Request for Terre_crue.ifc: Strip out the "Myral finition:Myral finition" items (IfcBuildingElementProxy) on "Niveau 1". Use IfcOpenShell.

First a look at what the model holds.

```python
import ifcopenshell
import ifcopenshell.util.element

model = ifcopenshell.open("Terre_crue.ifc")
print(model.schema)
storey = next(s for s in model.by_type("IfcBuildingStorey") if s.Name == "Niveau 1")
proxies = [e for e in ifcopenshell.util.element.get_decomposition(storey) if e.is_a("IfcBuildingElementProxy")]
seen = {}
for e in proxies:
    element_type = ifcopenshell.util.element.get_type(e)
    name = element_type.Name if element_type not in (None, e) else None
    seen[name] = seen.get(name, 0) + 1
for name, count in sorted(seen.items(), key=str):
    print(count, "x", name)
```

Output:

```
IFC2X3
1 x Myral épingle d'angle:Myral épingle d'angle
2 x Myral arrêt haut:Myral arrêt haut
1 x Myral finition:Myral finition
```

```python
import ifcopenshell
import ifcopenshell.api.root
import ifcopenshell.util.element

model = ifcopenshell.open("Terre_crue.ifc")

storey = next(s for s in model.by_type("IfcBuildingStorey") if s.Name == "Niveau 1")
proxies = [e for e in ifcopenshell.util.element.get_decomposition(storey) if e.is_a("IfcBuildingElementProxy")]
targets = [e for e in proxies if (t := ifcopenshell.util.element.get_type(e)) not in (None, e) and t.Name == "Myral finition:Myral finition"]

for e in targets:
    ifcopenshell.api.root.remove_product(model, product=e)
print(len(targets), "removed")

model.write("Terre_crue-out.ifc")
```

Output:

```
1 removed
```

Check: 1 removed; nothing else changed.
